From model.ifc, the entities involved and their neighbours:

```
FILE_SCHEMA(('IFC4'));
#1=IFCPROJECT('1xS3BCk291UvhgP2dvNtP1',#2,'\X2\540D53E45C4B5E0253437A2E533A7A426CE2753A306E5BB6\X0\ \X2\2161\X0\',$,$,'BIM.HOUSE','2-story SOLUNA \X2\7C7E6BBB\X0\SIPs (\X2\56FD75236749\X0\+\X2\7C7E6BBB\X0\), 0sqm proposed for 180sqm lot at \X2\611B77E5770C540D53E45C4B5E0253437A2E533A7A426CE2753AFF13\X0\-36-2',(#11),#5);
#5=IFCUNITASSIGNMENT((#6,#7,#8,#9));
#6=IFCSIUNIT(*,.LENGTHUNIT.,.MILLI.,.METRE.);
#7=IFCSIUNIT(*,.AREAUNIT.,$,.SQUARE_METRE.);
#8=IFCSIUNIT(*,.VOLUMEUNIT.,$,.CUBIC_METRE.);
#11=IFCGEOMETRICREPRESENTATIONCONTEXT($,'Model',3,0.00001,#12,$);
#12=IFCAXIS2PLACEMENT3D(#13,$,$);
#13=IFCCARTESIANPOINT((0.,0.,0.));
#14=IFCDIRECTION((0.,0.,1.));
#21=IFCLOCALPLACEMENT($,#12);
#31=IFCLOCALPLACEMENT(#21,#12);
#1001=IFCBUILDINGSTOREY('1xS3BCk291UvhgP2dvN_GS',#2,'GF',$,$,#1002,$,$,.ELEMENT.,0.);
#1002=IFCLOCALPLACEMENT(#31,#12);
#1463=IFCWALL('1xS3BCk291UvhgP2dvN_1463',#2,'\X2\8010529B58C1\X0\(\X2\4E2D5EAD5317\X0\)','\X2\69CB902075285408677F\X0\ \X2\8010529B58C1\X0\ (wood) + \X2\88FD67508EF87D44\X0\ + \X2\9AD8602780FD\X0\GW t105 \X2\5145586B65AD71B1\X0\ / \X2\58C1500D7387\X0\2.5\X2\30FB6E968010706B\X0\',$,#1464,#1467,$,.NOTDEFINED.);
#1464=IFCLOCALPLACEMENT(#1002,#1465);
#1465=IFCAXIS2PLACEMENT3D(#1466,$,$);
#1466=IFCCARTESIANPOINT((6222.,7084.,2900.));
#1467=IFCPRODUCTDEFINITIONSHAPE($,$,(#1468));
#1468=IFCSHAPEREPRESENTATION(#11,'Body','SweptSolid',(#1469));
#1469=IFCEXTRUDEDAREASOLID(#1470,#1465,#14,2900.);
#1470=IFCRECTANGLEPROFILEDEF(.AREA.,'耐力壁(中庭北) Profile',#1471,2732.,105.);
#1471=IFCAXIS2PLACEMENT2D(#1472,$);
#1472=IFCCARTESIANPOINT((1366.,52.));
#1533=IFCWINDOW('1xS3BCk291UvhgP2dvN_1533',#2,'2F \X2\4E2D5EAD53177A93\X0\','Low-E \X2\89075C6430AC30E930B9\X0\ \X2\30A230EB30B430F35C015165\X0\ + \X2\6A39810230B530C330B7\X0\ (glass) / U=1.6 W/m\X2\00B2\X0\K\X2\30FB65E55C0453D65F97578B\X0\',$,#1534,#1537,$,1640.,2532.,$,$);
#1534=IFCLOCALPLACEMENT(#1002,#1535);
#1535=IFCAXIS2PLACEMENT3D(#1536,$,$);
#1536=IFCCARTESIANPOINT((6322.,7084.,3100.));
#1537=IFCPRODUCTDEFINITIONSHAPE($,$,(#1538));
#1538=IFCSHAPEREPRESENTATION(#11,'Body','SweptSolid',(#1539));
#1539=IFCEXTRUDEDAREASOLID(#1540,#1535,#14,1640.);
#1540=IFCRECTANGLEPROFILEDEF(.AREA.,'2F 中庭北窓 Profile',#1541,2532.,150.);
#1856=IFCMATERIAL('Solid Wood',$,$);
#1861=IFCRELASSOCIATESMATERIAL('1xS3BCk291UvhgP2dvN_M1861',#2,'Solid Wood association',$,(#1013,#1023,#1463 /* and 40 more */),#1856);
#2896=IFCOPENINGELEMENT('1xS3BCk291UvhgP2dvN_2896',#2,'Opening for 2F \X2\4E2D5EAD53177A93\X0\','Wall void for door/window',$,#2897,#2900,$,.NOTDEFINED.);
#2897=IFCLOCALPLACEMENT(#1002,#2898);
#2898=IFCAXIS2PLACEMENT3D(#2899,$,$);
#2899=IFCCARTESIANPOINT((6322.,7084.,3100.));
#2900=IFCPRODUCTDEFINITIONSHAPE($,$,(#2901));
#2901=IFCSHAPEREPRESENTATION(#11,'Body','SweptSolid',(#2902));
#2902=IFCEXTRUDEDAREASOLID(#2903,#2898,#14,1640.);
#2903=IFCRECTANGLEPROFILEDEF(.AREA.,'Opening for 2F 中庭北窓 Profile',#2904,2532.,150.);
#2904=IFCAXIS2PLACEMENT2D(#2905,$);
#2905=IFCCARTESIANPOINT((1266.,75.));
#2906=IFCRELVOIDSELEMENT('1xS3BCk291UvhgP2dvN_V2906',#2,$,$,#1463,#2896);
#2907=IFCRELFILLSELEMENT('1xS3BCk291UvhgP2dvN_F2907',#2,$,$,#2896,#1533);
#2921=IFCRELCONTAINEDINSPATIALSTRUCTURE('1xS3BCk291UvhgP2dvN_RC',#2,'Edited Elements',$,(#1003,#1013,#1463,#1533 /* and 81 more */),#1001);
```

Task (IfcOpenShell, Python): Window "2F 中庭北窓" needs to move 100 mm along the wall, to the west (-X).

```python
import ifcopenshell
import ifcopenshell.api.geometry
import ifcopenshell.util.placement

model = ifcopenshell.open("model.ifc")

window = model.by_guid("1xS3BCk291UvhgP2dvN_1533")
opening = window.FillsVoids[0].RelatingOpeningElement
wall = opening.VoidsElements[0].RelatingBuildingElement

wall_matrix = ifcopenshell.util.placement.get_local_placement(wall.ObjectPlacement)
shift = wall_matrix[:3, 0] * -100.0
before = ifcopenshell.util.placement.get_local_placement(window.ObjectPlacement)[:3, 3].copy()

# The window is not placed relative to its opening, so move both.
for product in (opening, window):
    matrix = ifcopenshell.util.placement.get_local_placement(product.ObjectPlacement)
    matrix[:3, 3] += shift
    ifcopenshell.api.geometry.edit_object_placement(model, product=product, matrix=matrix, is_si=False)

after = ifcopenshell.util.placement.get_local_placement(window.ObjectPlacement)[:3, 3]
print("window moved by", (after - before).round(3) + 0.0)

model.write("model_edited.ifc")
```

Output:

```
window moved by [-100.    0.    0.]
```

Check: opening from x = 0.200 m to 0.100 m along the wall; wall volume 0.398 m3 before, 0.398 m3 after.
